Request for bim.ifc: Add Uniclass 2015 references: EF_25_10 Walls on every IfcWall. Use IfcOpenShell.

First a look at what the model holds.

```python
import ifcopenshell

model = ifcopenshell.open("bim.ifc")
print(model.schema)
print("classifications:", [c.Name for c in model.by_type("IfcClassification")])
for ifc_class in ("IfcDoor", "IfcRoof", "IfcStair", "IfcWall", "IfcWindow"):
    print(ifc_class, len(model.by_type(ifc_class)))
```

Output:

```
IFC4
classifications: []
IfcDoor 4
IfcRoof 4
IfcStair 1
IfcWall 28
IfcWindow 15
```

```python
import ifcopenshell
import ifcopenshell.api.classification

model = ifcopenshell.open("bim.ifc")

system = ifcopenshell.api.classification.add_classification(model, classification="Uniclass 2015")

codes = {
    "IfcWall": ("EF_25_10", "Walls"),
}
for ifc_class, (code, name) in codes.items():
    products = model.by_type(ifc_class)
    ifcopenshell.api.classification.add_reference(
        model, products=products, classification=system, identification=code, name=name
    )
    print(code, len(products))

model.write("bim-out.ifc")
```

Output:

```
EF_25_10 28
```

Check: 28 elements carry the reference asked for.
